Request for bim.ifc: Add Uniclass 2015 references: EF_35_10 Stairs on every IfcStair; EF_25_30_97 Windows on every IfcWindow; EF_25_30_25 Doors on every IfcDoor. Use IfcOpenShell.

First a look at what the model holds.

```python
import ifcopenshell

model = ifcopenshell.open("bim.ifc")
print(model.schema)
print("classifications:", [c.Name for c in model.by_type("IfcClassification")])
for ifc_class in ("IfcDoor", "IfcRoof", "IfcStair", "IfcWall", "IfcWindow"):
    print(ifc_class, len(model.by_type(ifc_class)))
```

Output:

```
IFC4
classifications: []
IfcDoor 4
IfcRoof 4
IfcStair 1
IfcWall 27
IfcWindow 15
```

```python
import ifcopenshell
import ifcopenshell.api.classification

model = ifcopenshell.open("bim.ifc")

system = ifcopenshell.api.classification.add_classification(model, classification="Uniclass 2015")

codes = {
    "IfcStair": ("EF_35_10", "Stairs"),
    "IfcWindow": ("EF_25_30_97", "Windows"),
    "IfcDoor": ("EF_25_30_25", "Doors"),
}
for ifc_class, (code, name) in codes.items():
    products = model.by_type(ifc_class)
    ifcopenshell.api.classification.add_reference(
        model, products=products, classification=system, identification=code, name=name
    )
    print(code, len(products))

model.write("bim_updated.ifc")
```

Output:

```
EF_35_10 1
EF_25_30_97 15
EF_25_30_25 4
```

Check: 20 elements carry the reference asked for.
